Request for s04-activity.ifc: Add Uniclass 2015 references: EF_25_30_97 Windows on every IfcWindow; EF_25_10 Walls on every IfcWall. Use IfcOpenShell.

First a look at what the model holds.

```python
import ifcopenshell

model = ifcopenshell.open("s04-activity.ifc")
print(model.schema)
print("classifications:", [c.Name for c in model.by_type("IfcClassification")])
for ifc_class in ("IfcDoor", "IfcRoof", "IfcStair", "IfcWall", "IfcWindow"):
    print(ifc_class, len(model.by_type(ifc_class)))
```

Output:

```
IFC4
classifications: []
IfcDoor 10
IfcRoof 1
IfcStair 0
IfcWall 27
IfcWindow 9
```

```python
import ifcopenshell
import ifcopenshell.api.classification

model = ifcopenshell.open("s04-activity.ifc")

system = ifcopenshell.api.classification.add_classification(model, classification="Uniclass 2015")

codes = {
    "IfcWindow": ("EF_25_30_97", "Windows"),
    "IfcWall": ("EF_25_10", "Walls"),
}
for ifc_class, (code, name) in codes.items():
    products = model.by_type(ifc_class)
    ifcopenshell.api.classification.add_reference(
        model, products=products, classification=system, identification=code, name=name
    )
    print(code, len(products))

model.write("s04-activity_edited.ifc")
```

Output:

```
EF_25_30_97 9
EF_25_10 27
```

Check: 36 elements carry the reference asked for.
